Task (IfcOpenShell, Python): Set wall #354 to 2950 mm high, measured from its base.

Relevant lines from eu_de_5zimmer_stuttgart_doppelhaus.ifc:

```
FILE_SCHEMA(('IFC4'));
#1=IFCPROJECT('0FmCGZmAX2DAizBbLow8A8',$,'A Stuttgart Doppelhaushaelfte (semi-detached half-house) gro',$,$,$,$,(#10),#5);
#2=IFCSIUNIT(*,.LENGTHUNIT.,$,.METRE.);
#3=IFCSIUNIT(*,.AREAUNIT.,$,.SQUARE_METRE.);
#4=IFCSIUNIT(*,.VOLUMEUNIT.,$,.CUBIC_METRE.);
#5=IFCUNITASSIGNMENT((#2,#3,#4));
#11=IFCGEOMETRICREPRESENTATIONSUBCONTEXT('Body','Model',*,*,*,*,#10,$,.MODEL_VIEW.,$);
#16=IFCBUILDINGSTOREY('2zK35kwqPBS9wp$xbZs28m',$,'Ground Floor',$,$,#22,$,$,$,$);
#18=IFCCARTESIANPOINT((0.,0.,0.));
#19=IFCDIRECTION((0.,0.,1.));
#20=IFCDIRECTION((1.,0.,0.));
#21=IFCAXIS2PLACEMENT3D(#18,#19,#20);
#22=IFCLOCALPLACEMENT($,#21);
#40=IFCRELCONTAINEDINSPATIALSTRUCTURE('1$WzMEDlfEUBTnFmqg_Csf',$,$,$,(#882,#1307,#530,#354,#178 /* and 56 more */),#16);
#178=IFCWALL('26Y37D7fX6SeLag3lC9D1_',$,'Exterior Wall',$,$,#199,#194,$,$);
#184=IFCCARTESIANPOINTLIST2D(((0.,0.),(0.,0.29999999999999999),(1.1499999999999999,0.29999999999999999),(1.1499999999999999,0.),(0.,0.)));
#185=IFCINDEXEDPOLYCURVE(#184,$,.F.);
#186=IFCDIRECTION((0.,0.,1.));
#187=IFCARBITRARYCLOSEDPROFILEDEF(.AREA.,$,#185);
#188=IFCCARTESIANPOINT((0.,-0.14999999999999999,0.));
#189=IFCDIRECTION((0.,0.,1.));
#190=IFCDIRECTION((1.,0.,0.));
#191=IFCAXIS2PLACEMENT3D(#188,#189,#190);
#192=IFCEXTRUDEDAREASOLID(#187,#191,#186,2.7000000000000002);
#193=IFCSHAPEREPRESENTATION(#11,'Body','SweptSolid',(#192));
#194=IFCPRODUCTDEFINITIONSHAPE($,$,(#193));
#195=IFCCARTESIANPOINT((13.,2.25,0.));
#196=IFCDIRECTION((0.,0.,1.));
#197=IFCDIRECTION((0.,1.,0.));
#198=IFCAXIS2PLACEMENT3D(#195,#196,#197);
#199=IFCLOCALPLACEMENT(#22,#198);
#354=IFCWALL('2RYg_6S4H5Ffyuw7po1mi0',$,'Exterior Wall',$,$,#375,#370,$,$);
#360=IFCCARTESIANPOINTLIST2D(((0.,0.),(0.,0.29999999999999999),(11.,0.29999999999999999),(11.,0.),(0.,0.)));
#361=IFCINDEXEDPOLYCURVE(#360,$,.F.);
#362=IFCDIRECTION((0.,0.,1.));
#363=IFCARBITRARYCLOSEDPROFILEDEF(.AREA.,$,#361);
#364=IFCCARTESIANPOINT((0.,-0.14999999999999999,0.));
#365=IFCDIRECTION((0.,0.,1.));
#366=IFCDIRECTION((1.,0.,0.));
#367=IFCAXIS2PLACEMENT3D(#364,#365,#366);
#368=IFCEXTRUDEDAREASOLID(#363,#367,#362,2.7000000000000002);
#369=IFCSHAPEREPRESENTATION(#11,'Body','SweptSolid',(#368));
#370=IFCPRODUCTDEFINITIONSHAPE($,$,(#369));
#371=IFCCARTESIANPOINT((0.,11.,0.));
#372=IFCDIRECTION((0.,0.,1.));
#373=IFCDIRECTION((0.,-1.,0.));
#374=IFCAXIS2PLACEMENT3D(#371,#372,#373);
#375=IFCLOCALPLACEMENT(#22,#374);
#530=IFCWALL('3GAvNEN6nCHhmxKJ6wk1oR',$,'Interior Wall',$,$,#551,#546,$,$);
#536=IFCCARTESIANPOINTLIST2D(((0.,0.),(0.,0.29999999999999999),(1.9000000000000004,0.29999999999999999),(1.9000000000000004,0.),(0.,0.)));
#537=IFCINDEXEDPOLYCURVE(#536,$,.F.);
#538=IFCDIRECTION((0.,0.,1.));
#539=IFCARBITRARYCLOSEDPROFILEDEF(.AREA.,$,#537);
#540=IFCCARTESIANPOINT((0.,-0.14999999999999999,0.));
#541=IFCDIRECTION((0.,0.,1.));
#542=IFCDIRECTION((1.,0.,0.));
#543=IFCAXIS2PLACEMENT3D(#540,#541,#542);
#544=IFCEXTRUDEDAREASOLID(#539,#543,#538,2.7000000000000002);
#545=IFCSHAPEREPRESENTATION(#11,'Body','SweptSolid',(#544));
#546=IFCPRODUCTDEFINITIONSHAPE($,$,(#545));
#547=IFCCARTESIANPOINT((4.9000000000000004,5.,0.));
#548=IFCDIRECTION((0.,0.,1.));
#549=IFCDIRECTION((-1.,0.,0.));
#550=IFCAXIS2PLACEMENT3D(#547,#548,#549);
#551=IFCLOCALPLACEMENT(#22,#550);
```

```python
import ifcopenshell
import ifcopenshell.geom
import ifcopenshell.util.representation
import ifcopenshell.util.shape

model = ifcopenshell.open("eu_de_5zimmer_stuttgart_doppelhaus.ifc")
settings = ifcopenshell.geom.settings()


def volume(element):
    """Net volume in cubic metres, openings subtracted."""
    shape = ifcopenshell.geom.create_shape(settings, element)
    return ifcopenshell.util.shape.get_volume(shape.geometry)


wall = model.by_guid("2RYg_6S4H5Ffyuw7po1mi0")
before = volume(wall)

body = ifcopenshell.util.representation.get_representation(wall, "Model", "Body")
solid = body.Items[0]
old_height = solid.Depth
solid.Depth = 2.95
after = volume(wall)

print(f"height {old_height:g} -> {solid.Depth:g}, volume {before:.3f} -> {after:.3f} m3")

model.write("eu_de_5zimmer_stuttgart_doppelhaus_rev.ifc")
```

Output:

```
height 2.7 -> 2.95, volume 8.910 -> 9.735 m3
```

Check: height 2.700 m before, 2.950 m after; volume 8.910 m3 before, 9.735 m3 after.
